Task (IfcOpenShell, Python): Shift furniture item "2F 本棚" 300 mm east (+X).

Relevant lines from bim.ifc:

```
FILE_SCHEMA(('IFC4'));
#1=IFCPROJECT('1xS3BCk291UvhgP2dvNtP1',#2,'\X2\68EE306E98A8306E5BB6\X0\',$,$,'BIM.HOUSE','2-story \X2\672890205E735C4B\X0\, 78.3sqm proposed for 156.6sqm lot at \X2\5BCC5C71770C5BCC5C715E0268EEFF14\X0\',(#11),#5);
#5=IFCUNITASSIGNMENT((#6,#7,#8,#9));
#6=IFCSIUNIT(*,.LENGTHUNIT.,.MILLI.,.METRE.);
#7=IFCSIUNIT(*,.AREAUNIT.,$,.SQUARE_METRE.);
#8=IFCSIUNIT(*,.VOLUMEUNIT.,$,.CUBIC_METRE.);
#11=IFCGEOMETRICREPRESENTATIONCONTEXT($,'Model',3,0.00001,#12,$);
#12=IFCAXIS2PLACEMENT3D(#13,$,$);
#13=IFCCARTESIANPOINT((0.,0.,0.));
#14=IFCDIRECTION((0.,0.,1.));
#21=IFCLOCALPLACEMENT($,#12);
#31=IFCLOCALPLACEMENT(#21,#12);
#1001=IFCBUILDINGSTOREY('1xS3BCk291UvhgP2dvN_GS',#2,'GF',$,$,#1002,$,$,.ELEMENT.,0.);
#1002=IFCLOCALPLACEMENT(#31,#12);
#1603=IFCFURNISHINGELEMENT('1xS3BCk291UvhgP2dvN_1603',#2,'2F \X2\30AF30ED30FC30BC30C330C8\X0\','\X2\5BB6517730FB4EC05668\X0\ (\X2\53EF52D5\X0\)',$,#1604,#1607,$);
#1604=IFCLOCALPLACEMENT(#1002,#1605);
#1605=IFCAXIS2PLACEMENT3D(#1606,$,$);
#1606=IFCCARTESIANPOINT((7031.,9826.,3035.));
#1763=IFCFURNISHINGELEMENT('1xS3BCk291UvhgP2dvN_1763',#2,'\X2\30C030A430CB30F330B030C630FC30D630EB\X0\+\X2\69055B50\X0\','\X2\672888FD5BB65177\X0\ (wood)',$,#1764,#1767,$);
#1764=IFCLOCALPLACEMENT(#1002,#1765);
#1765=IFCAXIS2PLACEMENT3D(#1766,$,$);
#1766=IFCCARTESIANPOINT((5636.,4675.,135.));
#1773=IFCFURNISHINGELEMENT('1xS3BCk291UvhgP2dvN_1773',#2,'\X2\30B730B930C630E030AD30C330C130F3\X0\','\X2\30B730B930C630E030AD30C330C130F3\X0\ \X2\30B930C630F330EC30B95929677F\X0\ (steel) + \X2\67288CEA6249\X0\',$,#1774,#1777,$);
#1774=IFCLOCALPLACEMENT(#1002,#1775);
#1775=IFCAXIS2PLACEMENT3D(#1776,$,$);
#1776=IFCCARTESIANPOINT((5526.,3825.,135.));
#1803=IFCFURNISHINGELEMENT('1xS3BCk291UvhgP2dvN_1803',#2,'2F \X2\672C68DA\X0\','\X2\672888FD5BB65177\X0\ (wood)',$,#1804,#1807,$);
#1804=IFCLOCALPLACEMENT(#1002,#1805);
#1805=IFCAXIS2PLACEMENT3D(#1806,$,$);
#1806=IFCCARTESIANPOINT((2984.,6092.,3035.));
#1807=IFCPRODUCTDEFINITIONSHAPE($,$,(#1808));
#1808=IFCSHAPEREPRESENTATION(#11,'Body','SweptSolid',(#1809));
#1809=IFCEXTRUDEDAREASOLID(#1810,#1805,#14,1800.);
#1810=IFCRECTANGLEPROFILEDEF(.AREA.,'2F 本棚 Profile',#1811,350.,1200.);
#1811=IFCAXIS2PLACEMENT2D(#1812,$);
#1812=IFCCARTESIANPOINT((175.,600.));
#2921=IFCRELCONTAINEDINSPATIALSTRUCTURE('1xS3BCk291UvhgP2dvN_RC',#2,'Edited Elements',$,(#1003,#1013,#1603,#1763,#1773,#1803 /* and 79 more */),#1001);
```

```python
import ifcopenshell
import ifcopenshell.api.geometry
import ifcopenshell.util.placement
import ifcopenshell.util.unit

model = ifcopenshell.open("bim.ifc")
unit_scale = ifcopenshell.util.unit.calculate_unit_scale(model)

item = model.by_guid("1xS3BCk291UvhgP2dvN_1803")
matrix = ifcopenshell.util.placement.get_local_placement(item.ObjectPlacement)
matrix[0, 3] += 0.3 / unit_scale
ifcopenshell.api.geometry.edit_object_placement(model, product=item, matrix=matrix, is_si=False)

print(ifcopenshell.util.placement.get_local_placement(item.ObjectPlacement).round(3) + 0.0)

model.write("bim_rev.ifc")
```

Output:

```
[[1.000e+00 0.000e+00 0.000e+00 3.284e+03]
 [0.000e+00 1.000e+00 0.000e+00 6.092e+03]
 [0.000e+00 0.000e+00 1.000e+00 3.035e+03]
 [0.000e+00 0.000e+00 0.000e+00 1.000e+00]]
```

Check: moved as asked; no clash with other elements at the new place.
